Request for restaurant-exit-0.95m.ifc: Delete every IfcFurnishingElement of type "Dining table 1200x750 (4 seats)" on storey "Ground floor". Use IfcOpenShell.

First a look at what the model holds.

```python
import ifcopenshell
import ifcopenshell.util.element

model = ifcopenshell.open("restaurant-exit-0.95m.ifc")
print(model.schema)
storey = next(s for s in model.by_type("IfcBuildingStorey") if s.Name == "Ground floor")
furniture = [e for e in ifcopenshell.util.element.get_decomposition(storey) if e.is_a("IfcFurnishingElement")]
seen = {}
for e in furniture:
    element_type = ifcopenshell.util.element.get_type(e)
    name = element_type.Name if element_type not in (None, e) else None
    seen[name] = seen.get(name, 0) + 1
for name, count in sorted(seen.items(), key=str):
    print(count, "x", name)
```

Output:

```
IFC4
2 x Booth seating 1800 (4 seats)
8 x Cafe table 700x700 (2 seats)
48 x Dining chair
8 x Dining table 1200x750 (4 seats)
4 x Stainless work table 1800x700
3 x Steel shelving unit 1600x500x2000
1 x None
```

```python
import ifcopenshell
import ifcopenshell.api.root
import ifcopenshell.util.element

model = ifcopenshell.open("restaurant-exit-0.95m.ifc")

storey = next(s for s in model.by_type("IfcBuildingStorey") if s.Name == "Ground floor")
furniture = [e for e in ifcopenshell.util.element.get_decomposition(storey) if e.is_a("IfcFurnishingElement")]
targets = [e for e in furniture if (t := ifcopenshell.util.element.get_type(e)) not in (None, e) and t.Name == "Dining table 1200x750 (4 seats)"]

for e in targets:
    ifcopenshell.api.root.remove_product(model, product=e)
print(len(targets), "removed")

model.write("restaurant-exit-0.95m-out.ifc")
```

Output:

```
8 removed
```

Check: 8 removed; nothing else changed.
